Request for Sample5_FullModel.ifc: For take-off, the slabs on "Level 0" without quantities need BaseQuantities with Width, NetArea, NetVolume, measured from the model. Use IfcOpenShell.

First a look at what the model holds.

```python
import ifcopenshell
import ifcopenshell.util.element
import ifcopenshell.util.unit

model = ifcopenshell.open("Sample5_FullModel.ifc")
print(model.schema)
for unit_type in ("LENGTHUNIT", "AREAUNIT", "VOLUMEUNIT"):
    print(unit_type, ifcopenshell.util.unit.calculate_unit_scale(model, unit_type))
storey = next(s for s in model.by_type("IfcBuildingStorey") if s.Name == "Level 0")
slabs = [e for e in ifcopenshell.util.element.get_decomposition(storey) if e.is_a("IfcSlab")]
for e in sorted(slabs, key=lambda e: e.id()):
    print(e.id(), e.is_a(), e.Name, list(ifcopenshell.util.element.get_psets(e, qtos_only=True)), sep=" | ")
```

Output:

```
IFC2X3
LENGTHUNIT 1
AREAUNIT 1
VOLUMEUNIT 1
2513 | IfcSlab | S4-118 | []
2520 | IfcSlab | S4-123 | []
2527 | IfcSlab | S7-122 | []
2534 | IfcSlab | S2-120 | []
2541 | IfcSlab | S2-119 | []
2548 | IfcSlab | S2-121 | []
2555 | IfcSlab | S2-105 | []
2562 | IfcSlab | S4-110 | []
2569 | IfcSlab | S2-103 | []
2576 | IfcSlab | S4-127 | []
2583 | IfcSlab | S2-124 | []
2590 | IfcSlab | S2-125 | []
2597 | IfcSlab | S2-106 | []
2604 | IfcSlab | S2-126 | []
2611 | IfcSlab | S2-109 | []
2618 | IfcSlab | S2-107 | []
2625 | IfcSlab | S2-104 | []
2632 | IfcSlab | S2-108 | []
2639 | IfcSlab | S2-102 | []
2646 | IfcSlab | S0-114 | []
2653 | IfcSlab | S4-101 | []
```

```python
import ifcopenshell
import ifcopenshell.api.pset
import ifcopenshell.geom
import ifcopenshell.util.element
import ifcopenshell.util.shape
import ifcopenshell.util.unit

model = ifcopenshell.open("Sample5_FullModel.ifc")
unit_scale = ifcopenshell.util.unit.calculate_unit_scale(model)
area_scale = ifcopenshell.util.unit.calculate_unit_scale(model, "AREAUNIT")
volume_scale = ifcopenshell.util.unit.calculate_unit_scale(model, "VOLUMEUNIT")
settings = ifcopenshell.geom.settings()

storey = next(s for s in model.by_type("IfcBuildingStorey") if s.Name == "Level 0")
slabs = [e for e in ifcopenshell.util.element.get_decomposition(storey) if e.is_a("IfcSlab")]

for e in sorted(slabs, key=lambda e: e.id()):
    if ifcopenshell.util.element.get_psets(e, qtos_only=True, should_inherit=False):
        continue
    # Geometry comes back in metres, in the element's own axes.
    shape = ifcopenshell.geom.create_shape(settings, e)
    values = {
        "Width": ifcopenshell.util.shape.get_z(shape.geometry) / unit_scale,
        "NetArea": ifcopenshell.util.shape.get_footprint_area(shape.geometry) / area_scale,
        "NetVolume": ifcopenshell.util.shape.get_volume(shape.geometry) / volume_scale,
    }
    qto = ifcopenshell.api.pset.add_qto(model, product=e, name="BaseQuantities")
    ifcopenshell.api.pset.edit_qto(model, qto=qto, properties=values)
    print(e.id(), {k: round(v, 3) for k, v in values.items()})

model.write("Sample5_FullModel-out.ifc")
```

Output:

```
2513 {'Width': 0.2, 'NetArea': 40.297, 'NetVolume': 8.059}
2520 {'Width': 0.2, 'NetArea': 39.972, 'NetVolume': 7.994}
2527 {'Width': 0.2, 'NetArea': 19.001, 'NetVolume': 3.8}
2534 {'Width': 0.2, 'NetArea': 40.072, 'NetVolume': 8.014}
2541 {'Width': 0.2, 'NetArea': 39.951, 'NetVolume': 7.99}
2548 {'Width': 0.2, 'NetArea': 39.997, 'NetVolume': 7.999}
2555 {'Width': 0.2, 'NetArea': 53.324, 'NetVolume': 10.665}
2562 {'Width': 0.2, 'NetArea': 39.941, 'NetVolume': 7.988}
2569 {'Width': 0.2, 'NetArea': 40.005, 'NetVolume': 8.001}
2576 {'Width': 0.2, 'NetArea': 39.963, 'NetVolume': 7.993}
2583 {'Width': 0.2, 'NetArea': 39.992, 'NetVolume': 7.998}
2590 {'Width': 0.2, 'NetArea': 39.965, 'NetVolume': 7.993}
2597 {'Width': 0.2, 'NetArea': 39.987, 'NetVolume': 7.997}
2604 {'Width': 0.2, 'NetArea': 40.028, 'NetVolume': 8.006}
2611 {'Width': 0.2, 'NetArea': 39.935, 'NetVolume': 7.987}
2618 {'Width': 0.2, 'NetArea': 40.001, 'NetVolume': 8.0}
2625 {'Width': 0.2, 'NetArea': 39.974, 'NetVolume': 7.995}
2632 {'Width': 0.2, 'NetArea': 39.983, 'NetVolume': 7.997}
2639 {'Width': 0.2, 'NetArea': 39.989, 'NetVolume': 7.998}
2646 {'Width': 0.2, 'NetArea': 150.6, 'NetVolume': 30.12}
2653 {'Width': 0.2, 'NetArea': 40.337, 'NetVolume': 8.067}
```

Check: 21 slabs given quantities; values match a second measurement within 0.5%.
